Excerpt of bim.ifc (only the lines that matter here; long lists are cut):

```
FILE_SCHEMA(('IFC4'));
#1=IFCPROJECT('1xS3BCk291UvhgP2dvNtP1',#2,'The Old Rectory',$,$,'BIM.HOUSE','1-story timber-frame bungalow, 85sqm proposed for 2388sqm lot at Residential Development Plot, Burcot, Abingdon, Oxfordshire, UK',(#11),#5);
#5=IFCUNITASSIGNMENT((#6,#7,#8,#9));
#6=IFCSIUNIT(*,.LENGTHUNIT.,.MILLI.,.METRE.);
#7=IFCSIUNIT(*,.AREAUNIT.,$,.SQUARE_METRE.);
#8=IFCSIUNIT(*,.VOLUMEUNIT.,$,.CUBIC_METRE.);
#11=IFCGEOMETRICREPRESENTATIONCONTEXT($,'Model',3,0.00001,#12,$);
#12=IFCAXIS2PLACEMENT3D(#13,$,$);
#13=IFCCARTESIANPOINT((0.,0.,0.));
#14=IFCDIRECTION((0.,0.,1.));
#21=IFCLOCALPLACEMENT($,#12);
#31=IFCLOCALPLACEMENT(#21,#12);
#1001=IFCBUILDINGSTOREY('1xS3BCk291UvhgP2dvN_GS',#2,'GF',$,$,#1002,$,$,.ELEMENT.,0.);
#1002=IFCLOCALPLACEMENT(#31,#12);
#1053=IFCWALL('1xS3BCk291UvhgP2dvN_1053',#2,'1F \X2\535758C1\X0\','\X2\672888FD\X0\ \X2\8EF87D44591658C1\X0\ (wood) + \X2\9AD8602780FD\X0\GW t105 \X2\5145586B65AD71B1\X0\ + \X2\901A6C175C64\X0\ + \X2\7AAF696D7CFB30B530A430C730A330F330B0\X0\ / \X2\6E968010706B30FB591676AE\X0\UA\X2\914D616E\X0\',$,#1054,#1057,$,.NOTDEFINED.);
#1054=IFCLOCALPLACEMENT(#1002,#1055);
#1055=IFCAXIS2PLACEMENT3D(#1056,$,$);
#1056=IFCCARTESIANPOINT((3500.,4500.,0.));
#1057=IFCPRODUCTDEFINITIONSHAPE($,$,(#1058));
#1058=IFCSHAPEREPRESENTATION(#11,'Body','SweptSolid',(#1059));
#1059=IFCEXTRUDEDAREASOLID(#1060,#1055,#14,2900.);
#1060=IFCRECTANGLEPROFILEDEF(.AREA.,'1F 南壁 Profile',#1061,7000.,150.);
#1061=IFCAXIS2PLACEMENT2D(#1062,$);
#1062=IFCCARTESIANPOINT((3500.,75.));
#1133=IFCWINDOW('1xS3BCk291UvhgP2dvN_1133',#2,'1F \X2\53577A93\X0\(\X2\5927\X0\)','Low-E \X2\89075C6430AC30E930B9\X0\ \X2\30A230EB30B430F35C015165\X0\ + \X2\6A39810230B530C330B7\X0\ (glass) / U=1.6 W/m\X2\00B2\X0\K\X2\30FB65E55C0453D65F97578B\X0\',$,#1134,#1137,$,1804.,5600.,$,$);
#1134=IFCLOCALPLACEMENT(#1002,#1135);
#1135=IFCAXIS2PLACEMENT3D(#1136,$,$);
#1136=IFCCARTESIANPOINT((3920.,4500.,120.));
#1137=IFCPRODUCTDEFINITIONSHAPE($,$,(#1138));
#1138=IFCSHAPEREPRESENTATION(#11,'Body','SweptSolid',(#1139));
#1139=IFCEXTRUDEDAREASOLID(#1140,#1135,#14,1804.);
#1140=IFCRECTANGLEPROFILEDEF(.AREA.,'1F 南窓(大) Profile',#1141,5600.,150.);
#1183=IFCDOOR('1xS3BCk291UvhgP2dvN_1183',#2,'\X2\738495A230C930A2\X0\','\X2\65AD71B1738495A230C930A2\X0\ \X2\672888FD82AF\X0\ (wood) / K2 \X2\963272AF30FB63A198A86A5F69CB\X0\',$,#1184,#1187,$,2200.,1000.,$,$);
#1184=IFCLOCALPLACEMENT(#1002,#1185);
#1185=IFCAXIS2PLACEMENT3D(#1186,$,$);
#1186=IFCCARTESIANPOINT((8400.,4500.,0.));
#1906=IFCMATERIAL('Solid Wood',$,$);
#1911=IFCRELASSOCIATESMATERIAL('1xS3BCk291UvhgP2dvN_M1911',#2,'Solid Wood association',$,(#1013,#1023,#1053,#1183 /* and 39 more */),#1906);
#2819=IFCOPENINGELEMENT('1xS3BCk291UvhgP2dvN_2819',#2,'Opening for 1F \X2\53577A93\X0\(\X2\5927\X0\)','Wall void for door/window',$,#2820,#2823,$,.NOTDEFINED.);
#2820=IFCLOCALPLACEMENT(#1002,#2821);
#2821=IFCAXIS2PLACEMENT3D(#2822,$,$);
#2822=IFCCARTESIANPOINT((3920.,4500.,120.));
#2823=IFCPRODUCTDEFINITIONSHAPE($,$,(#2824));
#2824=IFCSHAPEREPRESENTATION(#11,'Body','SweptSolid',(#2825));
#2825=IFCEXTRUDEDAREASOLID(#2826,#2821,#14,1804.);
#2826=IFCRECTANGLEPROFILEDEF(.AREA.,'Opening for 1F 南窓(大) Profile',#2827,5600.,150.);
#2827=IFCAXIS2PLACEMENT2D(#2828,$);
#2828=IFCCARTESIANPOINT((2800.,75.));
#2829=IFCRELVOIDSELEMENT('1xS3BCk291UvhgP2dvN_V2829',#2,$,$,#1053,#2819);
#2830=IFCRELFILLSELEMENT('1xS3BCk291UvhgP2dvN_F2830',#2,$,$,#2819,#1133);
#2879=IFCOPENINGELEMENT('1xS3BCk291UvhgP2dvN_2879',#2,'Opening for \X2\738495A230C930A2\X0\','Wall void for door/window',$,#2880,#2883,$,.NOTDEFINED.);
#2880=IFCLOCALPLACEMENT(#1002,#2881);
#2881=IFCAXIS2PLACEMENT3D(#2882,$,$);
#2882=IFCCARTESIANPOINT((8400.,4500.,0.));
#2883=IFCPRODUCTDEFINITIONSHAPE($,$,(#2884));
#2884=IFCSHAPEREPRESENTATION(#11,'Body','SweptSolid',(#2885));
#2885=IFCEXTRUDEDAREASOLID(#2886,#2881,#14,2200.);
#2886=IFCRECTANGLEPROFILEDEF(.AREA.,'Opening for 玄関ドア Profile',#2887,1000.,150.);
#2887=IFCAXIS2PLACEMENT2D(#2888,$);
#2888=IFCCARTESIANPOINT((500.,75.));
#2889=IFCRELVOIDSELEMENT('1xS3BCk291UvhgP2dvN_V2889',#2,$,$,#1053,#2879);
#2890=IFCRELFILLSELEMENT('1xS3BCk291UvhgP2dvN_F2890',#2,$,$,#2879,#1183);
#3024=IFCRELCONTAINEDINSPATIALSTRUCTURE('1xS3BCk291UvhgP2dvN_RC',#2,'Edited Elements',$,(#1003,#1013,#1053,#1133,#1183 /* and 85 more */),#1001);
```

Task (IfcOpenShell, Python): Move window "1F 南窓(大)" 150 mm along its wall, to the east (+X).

```python
import ifcopenshell
import ifcopenshell.api.geometry
import ifcopenshell.util.placement
import ifcopenshell.util.unit

model = ifcopenshell.open("bim.ifc")
unit_scale = ifcopenshell.util.unit.calculate_unit_scale(model)

window = model.by_guid("1xS3BCk291UvhgP2dvN_1133")
opening = window.FillsVoids[0].RelatingOpeningElement
wall = opening.VoidsElements[0].RelatingBuildingElement

wall_matrix = ifcopenshell.util.placement.get_local_placement(wall.ObjectPlacement)
shift = wall_matrix[:3, 0] * 0.15 / unit_scale
before = ifcopenshell.util.placement.get_local_placement(window.ObjectPlacement)[:3, 3].copy()

# The window is not placed relative to its opening, so move both.
for product in (opening, window):
    matrix = ifcopenshell.util.placement.get_local_placement(product.ObjectPlacement)
    matrix[:3, 3] += shift
    ifcopenshell.api.geometry.edit_object_placement(model, product=product, matrix=matrix, is_si=False)

after = ifcopenshell.util.placement.get_local_placement(window.ObjectPlacement)[:3, 3]
print("window moved by", (after - before).round(3) + 0.0)

model.write("bim_updated.ifc")
```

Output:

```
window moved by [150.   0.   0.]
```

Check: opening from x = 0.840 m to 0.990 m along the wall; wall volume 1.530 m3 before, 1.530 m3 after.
